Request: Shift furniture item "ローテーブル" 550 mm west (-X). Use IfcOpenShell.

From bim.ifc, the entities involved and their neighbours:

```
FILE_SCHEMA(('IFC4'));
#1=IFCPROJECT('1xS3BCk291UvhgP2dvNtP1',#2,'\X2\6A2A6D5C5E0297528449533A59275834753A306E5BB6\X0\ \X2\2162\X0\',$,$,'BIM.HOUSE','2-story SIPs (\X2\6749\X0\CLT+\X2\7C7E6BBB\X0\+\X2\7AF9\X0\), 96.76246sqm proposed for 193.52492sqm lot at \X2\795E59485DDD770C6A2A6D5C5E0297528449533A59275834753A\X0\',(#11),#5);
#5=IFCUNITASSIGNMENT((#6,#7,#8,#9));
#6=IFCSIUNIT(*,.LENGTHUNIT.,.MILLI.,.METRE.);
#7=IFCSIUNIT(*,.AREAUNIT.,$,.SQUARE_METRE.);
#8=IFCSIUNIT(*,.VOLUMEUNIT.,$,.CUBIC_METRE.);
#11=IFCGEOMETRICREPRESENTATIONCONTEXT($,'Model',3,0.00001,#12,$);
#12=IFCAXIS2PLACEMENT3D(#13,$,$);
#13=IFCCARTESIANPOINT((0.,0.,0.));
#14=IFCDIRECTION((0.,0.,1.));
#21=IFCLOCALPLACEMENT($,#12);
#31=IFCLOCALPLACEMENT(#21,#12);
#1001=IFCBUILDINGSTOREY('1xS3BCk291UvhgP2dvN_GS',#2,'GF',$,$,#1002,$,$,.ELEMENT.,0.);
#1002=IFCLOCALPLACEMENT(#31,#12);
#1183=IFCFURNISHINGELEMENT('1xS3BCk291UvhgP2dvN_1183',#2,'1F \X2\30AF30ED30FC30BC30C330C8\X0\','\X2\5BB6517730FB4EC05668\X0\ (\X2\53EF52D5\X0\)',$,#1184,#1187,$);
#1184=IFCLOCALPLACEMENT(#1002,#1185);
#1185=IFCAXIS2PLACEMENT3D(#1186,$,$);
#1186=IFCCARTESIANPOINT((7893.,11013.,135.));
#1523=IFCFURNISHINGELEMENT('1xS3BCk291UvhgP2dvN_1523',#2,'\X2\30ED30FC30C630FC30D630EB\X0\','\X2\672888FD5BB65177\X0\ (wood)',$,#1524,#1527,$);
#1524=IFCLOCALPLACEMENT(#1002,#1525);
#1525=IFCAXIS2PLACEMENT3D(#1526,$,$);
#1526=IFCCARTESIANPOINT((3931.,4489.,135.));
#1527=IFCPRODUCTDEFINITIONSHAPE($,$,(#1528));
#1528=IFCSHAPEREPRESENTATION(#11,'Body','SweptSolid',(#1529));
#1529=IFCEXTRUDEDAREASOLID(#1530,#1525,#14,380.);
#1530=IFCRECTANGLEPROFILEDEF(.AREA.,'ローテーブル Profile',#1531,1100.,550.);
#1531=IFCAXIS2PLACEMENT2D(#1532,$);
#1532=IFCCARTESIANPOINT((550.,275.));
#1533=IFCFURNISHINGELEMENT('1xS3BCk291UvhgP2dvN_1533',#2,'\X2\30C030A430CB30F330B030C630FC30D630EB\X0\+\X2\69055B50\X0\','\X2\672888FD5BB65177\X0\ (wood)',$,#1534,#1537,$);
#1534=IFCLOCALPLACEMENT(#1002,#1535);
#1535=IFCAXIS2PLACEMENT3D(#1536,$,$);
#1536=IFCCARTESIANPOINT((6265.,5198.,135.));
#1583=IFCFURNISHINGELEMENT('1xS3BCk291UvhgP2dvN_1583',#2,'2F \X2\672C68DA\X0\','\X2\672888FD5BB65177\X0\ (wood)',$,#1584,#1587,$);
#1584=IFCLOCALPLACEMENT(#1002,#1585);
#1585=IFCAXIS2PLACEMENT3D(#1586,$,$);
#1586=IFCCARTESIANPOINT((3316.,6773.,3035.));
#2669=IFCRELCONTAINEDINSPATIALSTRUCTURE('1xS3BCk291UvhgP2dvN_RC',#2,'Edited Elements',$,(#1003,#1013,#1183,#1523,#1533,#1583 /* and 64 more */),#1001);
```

```python
import ifcopenshell
import ifcopenshell.api.geometry
import ifcopenshell.util.placement

model = ifcopenshell.open("bim.ifc")

item = model.by_guid("1xS3BCk291UvhgP2dvN_1523")
matrix = ifcopenshell.util.placement.get_local_placement(item.ObjectPlacement)
matrix[0, 3] -= 550.0
ifcopenshell.api.geometry.edit_object_placement(model, product=item, matrix=matrix, is_si=False)

print(ifcopenshell.util.placement.get_local_placement(item.ObjectPlacement).round(3) + 0.0)

model.write("bim_rev.ifc")
```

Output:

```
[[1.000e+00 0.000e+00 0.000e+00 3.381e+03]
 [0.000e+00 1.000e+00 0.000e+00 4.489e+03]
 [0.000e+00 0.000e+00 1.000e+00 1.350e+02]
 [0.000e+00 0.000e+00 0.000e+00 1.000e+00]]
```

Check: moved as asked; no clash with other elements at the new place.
